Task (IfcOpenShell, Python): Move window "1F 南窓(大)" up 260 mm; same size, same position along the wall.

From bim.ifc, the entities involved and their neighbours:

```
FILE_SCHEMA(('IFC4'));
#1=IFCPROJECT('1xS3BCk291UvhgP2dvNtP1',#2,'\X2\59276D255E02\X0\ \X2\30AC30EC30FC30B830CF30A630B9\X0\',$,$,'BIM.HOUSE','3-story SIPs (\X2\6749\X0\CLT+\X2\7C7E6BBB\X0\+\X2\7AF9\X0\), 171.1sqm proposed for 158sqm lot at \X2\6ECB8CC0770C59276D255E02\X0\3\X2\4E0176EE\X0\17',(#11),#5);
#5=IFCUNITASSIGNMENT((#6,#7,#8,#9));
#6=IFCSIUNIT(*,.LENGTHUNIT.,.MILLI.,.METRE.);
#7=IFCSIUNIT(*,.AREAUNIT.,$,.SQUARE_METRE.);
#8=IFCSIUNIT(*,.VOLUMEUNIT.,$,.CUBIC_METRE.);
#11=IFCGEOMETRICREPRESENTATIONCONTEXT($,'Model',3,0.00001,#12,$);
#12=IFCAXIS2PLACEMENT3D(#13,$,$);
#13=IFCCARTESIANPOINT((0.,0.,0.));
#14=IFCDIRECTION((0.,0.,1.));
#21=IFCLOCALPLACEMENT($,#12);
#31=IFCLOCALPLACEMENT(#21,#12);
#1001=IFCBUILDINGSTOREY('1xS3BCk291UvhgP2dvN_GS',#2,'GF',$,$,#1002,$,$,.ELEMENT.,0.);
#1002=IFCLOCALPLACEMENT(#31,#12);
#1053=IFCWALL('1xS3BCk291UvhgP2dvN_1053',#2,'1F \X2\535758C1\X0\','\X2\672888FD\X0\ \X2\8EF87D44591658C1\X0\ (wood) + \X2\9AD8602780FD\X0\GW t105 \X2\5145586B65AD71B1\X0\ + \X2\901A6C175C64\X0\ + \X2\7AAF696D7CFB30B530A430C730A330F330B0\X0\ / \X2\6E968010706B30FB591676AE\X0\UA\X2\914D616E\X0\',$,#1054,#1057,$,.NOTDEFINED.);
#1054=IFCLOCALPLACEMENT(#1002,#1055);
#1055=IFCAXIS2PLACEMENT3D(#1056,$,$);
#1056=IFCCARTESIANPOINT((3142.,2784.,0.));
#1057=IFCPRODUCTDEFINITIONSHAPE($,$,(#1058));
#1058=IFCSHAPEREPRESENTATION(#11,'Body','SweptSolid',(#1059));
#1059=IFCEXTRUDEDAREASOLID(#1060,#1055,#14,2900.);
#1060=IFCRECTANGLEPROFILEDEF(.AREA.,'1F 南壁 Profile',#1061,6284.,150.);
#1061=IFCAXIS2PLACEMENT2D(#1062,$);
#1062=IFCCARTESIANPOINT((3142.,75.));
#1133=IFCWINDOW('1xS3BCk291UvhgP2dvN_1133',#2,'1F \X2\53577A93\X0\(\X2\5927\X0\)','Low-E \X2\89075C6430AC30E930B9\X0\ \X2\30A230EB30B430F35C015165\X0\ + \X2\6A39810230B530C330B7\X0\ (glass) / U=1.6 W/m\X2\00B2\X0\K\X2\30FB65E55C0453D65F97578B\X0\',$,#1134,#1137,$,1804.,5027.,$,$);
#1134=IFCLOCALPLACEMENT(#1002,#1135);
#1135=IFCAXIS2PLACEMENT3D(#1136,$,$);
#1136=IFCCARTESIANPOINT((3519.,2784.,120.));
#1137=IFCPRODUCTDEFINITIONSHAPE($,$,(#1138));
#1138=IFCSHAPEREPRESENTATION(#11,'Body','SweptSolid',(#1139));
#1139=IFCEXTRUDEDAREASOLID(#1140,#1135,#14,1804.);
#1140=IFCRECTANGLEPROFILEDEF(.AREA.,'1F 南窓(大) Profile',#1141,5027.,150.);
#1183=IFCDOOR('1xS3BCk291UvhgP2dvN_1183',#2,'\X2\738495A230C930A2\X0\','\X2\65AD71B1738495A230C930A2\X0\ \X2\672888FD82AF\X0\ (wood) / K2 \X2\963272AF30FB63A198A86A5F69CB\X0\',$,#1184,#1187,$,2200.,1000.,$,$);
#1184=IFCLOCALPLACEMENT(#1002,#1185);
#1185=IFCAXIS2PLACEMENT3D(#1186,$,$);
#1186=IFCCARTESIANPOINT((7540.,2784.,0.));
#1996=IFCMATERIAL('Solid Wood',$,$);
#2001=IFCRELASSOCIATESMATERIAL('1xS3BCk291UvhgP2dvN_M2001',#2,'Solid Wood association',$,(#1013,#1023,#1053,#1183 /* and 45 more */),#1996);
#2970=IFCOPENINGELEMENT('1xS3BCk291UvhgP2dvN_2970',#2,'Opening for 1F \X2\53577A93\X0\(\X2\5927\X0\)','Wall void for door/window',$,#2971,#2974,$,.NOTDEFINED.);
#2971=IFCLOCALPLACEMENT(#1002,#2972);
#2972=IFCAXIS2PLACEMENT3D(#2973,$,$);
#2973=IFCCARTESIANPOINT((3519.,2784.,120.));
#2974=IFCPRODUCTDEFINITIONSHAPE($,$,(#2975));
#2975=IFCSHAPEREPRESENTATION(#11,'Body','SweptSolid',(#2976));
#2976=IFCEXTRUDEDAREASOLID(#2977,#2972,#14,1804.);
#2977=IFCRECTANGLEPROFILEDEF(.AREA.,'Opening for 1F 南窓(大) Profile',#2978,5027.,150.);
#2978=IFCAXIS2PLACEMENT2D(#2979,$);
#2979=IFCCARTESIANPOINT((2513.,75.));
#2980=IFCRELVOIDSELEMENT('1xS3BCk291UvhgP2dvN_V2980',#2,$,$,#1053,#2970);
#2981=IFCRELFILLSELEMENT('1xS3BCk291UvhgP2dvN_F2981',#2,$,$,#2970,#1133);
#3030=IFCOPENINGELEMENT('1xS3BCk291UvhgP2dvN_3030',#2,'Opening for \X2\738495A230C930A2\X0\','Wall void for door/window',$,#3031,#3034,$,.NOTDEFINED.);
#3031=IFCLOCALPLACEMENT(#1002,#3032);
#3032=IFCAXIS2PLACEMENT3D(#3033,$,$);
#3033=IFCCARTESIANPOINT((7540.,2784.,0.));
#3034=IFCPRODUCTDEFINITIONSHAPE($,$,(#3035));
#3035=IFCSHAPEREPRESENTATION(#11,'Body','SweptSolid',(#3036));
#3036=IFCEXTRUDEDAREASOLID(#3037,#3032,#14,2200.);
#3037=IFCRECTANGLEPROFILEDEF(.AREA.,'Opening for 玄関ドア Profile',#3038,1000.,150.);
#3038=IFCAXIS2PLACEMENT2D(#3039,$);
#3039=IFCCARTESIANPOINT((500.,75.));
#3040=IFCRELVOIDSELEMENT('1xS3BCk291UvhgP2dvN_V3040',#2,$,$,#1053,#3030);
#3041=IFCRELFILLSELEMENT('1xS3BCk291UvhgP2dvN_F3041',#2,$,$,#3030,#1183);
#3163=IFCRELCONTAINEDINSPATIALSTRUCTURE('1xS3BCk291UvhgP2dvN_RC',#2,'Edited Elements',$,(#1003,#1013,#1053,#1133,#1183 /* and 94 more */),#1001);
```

```python
import numpy as np
import ifcopenshell
import ifcopenshell.api.geometry
import ifcopenshell.util.placement
import ifcopenshell.util.unit

model = ifcopenshell.open("bim.ifc")
unit_scale = ifcopenshell.util.unit.calculate_unit_scale(model)

window = model.by_id(1133)
opening = window.FillsVoids[0].RelatingOpeningElement
dz = 0.26 / unit_scale

shift = np.array([0.0, 0.0, dz])
# The window is not placed relative to its opening, so move both.
for product in (opening, window):
    matrix = ifcopenshell.util.placement.get_local_placement(product.ObjectPlacement)
    matrix[:3, 3] += shift
    ifcopenshell.api.geometry.edit_object_placement(model, product=product, matrix=matrix, is_si=False)

print(f"moved by {dz * unit_scale:+.3f} m")

model.write("bim-out.ifc")
```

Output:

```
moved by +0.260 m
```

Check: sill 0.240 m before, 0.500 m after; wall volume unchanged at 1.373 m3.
